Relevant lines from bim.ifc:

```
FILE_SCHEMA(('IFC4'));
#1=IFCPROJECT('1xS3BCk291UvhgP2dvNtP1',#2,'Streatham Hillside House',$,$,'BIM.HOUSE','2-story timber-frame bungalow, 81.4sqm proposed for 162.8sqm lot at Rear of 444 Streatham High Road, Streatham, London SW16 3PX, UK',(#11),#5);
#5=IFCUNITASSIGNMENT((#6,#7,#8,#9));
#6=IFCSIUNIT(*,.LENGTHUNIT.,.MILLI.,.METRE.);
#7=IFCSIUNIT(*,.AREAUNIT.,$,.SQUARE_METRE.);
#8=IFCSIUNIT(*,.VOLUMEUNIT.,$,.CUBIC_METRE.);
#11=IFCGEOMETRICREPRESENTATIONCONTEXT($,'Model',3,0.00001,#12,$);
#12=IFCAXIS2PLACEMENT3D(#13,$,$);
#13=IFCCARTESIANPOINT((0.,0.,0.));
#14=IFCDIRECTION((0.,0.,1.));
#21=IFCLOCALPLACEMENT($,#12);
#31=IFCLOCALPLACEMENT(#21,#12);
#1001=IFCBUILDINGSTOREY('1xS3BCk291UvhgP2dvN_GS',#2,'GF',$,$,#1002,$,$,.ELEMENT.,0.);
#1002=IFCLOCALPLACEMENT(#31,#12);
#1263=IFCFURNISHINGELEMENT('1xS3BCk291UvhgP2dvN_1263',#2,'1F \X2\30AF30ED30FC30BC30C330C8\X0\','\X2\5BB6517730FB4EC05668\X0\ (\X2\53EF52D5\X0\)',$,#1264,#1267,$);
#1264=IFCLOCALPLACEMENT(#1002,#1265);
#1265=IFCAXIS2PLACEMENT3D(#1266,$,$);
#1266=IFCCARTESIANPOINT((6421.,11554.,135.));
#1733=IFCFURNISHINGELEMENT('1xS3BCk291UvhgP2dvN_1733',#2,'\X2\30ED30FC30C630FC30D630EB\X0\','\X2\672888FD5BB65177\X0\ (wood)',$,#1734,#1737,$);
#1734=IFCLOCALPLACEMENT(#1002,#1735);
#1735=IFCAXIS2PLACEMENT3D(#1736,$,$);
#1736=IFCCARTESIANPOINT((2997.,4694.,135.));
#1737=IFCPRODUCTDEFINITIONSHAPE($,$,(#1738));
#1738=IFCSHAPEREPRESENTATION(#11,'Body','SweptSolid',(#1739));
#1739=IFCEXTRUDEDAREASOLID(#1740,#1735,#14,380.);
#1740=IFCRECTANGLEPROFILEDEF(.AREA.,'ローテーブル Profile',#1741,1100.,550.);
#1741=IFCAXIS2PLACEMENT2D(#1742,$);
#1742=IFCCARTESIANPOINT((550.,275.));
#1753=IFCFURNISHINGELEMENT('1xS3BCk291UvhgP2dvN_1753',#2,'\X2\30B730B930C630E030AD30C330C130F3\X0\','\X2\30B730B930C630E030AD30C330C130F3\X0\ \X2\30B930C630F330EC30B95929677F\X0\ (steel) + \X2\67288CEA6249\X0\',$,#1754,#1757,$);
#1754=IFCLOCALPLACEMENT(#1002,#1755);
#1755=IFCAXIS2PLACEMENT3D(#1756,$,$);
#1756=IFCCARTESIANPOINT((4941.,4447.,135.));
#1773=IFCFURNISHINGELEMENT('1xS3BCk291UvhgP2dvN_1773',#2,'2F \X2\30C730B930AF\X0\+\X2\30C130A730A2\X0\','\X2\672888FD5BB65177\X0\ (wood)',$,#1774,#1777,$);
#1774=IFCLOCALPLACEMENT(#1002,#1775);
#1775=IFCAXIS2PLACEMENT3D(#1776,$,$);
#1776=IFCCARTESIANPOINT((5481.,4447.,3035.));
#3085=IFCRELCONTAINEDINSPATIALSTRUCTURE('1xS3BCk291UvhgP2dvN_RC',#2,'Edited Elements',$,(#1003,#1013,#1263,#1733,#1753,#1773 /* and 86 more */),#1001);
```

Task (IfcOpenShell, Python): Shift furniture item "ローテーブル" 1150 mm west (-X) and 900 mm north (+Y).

```python
import ifcopenshell
import ifcopenshell.api.geometry
import ifcopenshell.util.placement

model = ifcopenshell.open("bim.ifc")

item = model.by_id(1733)
matrix = ifcopenshell.util.placement.get_local_placement(item.ObjectPlacement)
matrix[0, 3] -= 1150.0
matrix[1, 3] += 900.0
ifcopenshell.api.geometry.edit_object_placement(model, product=item, matrix=matrix, is_si=False)

print(ifcopenshell.util.placement.get_local_placement(item.ObjectPlacement).round(3) + 0.0)

model.write("bim_edited.ifc")
```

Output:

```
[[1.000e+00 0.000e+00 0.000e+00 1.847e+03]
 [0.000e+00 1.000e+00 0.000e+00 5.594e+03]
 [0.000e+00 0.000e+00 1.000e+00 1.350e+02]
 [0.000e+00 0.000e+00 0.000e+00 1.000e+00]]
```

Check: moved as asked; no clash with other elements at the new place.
